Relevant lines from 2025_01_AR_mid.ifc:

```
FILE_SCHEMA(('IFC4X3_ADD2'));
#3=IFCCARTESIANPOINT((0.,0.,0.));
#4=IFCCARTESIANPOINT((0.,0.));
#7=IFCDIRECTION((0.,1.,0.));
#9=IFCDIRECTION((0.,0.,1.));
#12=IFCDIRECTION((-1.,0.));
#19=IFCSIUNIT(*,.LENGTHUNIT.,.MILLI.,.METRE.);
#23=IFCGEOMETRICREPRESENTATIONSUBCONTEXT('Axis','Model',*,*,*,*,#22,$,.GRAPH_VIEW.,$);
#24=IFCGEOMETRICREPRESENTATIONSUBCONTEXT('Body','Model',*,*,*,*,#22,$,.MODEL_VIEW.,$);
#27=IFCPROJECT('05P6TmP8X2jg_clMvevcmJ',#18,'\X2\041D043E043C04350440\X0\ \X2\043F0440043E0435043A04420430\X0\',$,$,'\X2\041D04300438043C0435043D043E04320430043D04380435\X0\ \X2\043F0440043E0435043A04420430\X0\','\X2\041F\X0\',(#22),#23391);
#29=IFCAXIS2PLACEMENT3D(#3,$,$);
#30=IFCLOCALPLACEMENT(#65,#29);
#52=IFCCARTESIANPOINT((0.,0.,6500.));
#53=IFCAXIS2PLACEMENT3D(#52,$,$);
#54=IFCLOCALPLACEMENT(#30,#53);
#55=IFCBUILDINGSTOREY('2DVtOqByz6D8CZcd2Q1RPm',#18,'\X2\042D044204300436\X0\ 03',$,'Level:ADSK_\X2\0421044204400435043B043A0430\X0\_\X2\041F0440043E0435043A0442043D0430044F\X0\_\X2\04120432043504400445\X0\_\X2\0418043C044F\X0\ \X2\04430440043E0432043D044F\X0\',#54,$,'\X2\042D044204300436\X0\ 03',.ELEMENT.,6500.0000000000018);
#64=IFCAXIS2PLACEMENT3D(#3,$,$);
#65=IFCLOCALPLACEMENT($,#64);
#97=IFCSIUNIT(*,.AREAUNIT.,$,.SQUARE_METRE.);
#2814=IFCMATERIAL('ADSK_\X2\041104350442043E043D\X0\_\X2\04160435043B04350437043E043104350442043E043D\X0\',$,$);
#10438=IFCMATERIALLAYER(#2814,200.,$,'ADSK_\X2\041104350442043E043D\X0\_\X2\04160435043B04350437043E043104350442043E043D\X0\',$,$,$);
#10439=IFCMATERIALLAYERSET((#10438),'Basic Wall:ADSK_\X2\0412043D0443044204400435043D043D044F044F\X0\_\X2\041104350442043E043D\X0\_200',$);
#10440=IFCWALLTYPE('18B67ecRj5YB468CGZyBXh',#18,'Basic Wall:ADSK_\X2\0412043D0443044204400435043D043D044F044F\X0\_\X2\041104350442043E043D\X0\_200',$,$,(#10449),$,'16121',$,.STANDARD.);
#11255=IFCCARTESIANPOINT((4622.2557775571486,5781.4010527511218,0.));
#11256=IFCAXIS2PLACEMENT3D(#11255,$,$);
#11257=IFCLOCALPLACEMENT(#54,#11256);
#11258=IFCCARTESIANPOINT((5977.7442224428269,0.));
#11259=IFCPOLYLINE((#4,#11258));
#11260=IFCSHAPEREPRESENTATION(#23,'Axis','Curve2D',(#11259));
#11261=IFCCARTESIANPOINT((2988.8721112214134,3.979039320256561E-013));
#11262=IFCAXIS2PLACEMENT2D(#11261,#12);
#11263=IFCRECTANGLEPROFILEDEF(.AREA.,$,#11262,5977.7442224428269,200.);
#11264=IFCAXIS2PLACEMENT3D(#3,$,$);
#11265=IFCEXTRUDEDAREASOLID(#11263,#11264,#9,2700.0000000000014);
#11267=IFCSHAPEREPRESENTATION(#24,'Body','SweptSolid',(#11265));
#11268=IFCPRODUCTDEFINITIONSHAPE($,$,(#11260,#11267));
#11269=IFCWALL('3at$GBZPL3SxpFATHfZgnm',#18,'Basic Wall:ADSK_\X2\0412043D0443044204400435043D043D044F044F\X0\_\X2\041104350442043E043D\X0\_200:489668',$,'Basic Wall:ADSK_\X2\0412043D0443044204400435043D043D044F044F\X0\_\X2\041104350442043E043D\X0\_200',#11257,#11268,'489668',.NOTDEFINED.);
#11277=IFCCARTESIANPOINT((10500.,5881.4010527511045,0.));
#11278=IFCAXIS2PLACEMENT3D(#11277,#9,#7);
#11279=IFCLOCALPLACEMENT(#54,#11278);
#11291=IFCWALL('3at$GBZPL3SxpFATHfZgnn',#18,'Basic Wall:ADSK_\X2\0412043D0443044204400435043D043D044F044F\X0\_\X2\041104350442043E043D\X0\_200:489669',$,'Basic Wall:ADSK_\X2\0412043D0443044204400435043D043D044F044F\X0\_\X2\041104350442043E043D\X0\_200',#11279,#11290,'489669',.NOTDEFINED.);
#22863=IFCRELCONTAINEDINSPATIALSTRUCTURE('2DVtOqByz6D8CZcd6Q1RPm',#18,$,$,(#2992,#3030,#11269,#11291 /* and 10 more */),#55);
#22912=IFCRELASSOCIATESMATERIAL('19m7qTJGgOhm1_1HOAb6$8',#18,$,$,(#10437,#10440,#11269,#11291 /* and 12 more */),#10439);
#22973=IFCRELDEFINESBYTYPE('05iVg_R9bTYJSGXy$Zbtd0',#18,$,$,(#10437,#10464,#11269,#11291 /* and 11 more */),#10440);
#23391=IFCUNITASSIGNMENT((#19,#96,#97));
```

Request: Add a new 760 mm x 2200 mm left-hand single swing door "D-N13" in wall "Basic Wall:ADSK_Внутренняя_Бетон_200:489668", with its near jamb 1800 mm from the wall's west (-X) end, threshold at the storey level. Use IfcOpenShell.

```python
import numpy as np
import ifcopenshell
import ifcopenshell.api.feature
import ifcopenshell.api.geometry
import ifcopenshell.api.root
import ifcopenshell.api.spatial
import ifcopenshell.geom
import ifcopenshell.util.element
import ifcopenshell.util.placement
import ifcopenshell.util.representation
import ifcopenshell.util.shape
import ifcopenshell.util.unit

model = ifcopenshell.open("2025_01_AR_mid.ifc")
unit_scale = ifcopenshell.util.unit.calculate_unit_scale(model)
settings = ifcopenshell.geom.settings()


def volume(element):
    """Net volume in cubic metres, openings subtracted."""
    shape = ifcopenshell.geom.create_shape(settings, element)
    return ifcopenshell.util.shape.get_volume(shape.geometry)


wall = model.by_guid("3at$GBZPL3SxpFATHfZgnm")
storey = ifcopenshell.util.element.get_container(wall, ifc_class="IfcBuildingStorey")
context = ifcopenshell.util.representation.get_context(model, "Model", "Body", "MODEL_VIEW")
before = volume(wall)

width, height, from_end, sill = 0.76, 2.2, 1.8, 0.0  # metres

# The wall runs along its own X axis, and the end named is its -X end.
wall_shape = ifcopenshell.geom.create_shape(settings, wall)
x, y, z = ifcopenshell.util.shape.get_vertices(wall_shape.geometry).T
start = x.min() + from_end
face, thickness = float(y.min()), float(y.max() - y.min())
wall_matrix = ifcopenshell.util.placement.get_local_placement(wall.ObjectPlacement)
level = ifcopenshell.util.placement.get_local_placement(storey.ObjectPlacement)[2, 3]


def in_wall(x, y):
    """Placement at x, y metres in the wall's axes, at sill height."""
    matrix = wall_matrix.copy()
    matrix[:, 3] = wall_matrix @ np.array([x / unit_scale, y / unit_scale, 0.0, 1.0])
    matrix[2, 3] = level + sill / unit_scale
    return matrix


# Opening: a box that overshoots both wall faces by 50 mm.
opening = ifcopenshell.api.root.create_entity(model, ifc_class="IfcOpeningElement", predefined_type="OPENING")
box = ifcopenshell.api.geometry.add_wall_representation(
    model, context=context, length=width, height=height, thickness=thickness + 0.1
)
ifcopenshell.api.geometry.assign_representation(model, product=opening, representation=box)
ifcopenshell.api.geometry.edit_object_placement(model, product=opening, matrix=in_wall(start, face - 0.05), is_si=False)
ifcopenshell.api.feature.add_feature(model, feature=opening, element=wall)

door = ifcopenshell.api.root.create_entity(model, ifc_class="IfcDoor", name="D-N13", predefined_type="DOOR")
door.OverallWidth, door.OverallHeight = width / unit_scale, height / unit_scale
door.OperationType = "SINGLE_SWING_LEFT"
body = ifcopenshell.api.geometry.add_door_representation(
    model,
    context=context,
    overall_width=door.OverallWidth,
    overall_height=door.OverallHeight,
    operation_type="SINGLE_SWING_LEFT",
    lining_properties={"LiningDepth": thickness / unit_scale, "ThresholdDepth": thickness / unit_scale},
)
ifcopenshell.api.geometry.assign_representation(model, product=door, representation=body)
ifcopenshell.api.spatial.assign_container(model, products=[door], relating_structure=storey)
ifcopenshell.api.feature.add_filling(model, opening=opening, element=door)

# The lining spans the wall, so the door starts at the wall face.
ifcopenshell.api.geometry.edit_object_placement(model, product=door, matrix=in_wall(start, face), is_si=False)

after = volume(wall)

print(f"wall volume {before:.3f} -> {after:.3f} m3")

model.write("2025_01_AR_mid_v2.ifc")
```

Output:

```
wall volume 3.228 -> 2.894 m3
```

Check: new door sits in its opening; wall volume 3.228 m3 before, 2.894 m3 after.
